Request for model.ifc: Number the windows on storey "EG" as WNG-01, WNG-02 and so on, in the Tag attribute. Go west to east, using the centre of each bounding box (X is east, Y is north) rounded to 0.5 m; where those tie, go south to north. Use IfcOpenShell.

First a look at what the model holds.

```python
import ifcopenshell
import ifcopenshell.util.element
import ifcopenshell.util.placement

model = ifcopenshell.open("model.ifc")
print(model.schema)
storey = next(s for s in model.by_type("IfcBuildingStorey") if s.Name == "EG")
windows = [e for e in ifcopenshell.util.element.get_decomposition(storey) if e.is_a("IfcWindow")]
for e in sorted(windows, key=lambda e: e.id()):
    origin = ifcopenshell.util.placement.get_local_placement(e.ObjectPlacement)[:3, 3]
    print(e.id(), e.Tag, e.Name, origin.round(2) + 0.0, sep=" | ")
```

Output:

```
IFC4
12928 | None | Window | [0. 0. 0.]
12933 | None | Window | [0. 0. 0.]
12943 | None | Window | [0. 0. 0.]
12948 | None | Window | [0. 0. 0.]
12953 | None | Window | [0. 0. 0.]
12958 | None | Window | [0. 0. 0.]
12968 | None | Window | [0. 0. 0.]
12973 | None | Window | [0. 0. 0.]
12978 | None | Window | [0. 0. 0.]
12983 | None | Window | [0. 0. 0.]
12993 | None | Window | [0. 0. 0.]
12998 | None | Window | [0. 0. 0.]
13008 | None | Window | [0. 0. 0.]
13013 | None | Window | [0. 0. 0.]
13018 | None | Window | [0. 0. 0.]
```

```python
import ifcopenshell
import ifcopenshell.geom
import ifcopenshell.util.element
import ifcopenshell.util.shape

model = ifcopenshell.open("model.ifc")
settings = ifcopenshell.geom.settings()
settings.set("use-world-coords", True)


def centre(element):
    shape = ifcopenshell.geom.create_shape(settings, element)
    return ifcopenshell.util.shape.get_bbox_centroid(shape.geometry)


storey = next(s for s in model.by_type("IfcBuildingStorey") if s.Name == "EG")
windows = [e for e in ifcopenshell.util.element.get_decomposition(storey) if e.is_a("IfcWindow")]

# Insertion points can sit at a corner or the storey origin, so sort by the geometry (in metres).
centres = {e: centre(e) for e in windows}
windows.sort(key=lambda e: (round(centres[e][0] / 0.5), centres[e][1]))

for i, e in enumerate(windows, start=1):
    number = f"WNG-{i:02d}"
    e.Tag = number
    print(e.id(), number)

model.write("model_v2.ifc")
```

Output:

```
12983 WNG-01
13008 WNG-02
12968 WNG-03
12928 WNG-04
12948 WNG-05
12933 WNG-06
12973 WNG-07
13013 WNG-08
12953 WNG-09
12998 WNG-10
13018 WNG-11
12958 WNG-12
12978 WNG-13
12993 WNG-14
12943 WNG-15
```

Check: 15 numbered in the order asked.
